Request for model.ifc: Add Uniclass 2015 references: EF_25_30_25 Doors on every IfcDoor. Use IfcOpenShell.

First a look at what the model holds.

```python
import ifcopenshell

model = ifcopenshell.open("model.ifc")
print(model.schema)
print("classifications:", [c.Name for c in model.by_type("IfcClassification")])
for ifc_class in ("IfcDoor", "IfcRoof", "IfcStair", "IfcWall", "IfcWindow"):
    print(ifc_class, len(model.by_type(ifc_class)))
```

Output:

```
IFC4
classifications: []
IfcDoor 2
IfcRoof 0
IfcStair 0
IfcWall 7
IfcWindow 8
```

```python
import ifcopenshell
import ifcopenshell.api.classification

model = ifcopenshell.open("model.ifc")

system = ifcopenshell.api.classification.add_classification(model, classification="Uniclass 2015")

codes = {
    "IfcDoor": ("EF_25_30_25", "Doors"),
}
for ifc_class, (code, name) in codes.items():
    products = model.by_type(ifc_class)
    ifcopenshell.api.classification.add_reference(
        model, products=products, classification=system, identification=code, name=name
    )
    print(code, len(products))

model.write("model_edited.ifc")
```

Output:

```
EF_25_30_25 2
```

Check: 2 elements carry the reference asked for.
